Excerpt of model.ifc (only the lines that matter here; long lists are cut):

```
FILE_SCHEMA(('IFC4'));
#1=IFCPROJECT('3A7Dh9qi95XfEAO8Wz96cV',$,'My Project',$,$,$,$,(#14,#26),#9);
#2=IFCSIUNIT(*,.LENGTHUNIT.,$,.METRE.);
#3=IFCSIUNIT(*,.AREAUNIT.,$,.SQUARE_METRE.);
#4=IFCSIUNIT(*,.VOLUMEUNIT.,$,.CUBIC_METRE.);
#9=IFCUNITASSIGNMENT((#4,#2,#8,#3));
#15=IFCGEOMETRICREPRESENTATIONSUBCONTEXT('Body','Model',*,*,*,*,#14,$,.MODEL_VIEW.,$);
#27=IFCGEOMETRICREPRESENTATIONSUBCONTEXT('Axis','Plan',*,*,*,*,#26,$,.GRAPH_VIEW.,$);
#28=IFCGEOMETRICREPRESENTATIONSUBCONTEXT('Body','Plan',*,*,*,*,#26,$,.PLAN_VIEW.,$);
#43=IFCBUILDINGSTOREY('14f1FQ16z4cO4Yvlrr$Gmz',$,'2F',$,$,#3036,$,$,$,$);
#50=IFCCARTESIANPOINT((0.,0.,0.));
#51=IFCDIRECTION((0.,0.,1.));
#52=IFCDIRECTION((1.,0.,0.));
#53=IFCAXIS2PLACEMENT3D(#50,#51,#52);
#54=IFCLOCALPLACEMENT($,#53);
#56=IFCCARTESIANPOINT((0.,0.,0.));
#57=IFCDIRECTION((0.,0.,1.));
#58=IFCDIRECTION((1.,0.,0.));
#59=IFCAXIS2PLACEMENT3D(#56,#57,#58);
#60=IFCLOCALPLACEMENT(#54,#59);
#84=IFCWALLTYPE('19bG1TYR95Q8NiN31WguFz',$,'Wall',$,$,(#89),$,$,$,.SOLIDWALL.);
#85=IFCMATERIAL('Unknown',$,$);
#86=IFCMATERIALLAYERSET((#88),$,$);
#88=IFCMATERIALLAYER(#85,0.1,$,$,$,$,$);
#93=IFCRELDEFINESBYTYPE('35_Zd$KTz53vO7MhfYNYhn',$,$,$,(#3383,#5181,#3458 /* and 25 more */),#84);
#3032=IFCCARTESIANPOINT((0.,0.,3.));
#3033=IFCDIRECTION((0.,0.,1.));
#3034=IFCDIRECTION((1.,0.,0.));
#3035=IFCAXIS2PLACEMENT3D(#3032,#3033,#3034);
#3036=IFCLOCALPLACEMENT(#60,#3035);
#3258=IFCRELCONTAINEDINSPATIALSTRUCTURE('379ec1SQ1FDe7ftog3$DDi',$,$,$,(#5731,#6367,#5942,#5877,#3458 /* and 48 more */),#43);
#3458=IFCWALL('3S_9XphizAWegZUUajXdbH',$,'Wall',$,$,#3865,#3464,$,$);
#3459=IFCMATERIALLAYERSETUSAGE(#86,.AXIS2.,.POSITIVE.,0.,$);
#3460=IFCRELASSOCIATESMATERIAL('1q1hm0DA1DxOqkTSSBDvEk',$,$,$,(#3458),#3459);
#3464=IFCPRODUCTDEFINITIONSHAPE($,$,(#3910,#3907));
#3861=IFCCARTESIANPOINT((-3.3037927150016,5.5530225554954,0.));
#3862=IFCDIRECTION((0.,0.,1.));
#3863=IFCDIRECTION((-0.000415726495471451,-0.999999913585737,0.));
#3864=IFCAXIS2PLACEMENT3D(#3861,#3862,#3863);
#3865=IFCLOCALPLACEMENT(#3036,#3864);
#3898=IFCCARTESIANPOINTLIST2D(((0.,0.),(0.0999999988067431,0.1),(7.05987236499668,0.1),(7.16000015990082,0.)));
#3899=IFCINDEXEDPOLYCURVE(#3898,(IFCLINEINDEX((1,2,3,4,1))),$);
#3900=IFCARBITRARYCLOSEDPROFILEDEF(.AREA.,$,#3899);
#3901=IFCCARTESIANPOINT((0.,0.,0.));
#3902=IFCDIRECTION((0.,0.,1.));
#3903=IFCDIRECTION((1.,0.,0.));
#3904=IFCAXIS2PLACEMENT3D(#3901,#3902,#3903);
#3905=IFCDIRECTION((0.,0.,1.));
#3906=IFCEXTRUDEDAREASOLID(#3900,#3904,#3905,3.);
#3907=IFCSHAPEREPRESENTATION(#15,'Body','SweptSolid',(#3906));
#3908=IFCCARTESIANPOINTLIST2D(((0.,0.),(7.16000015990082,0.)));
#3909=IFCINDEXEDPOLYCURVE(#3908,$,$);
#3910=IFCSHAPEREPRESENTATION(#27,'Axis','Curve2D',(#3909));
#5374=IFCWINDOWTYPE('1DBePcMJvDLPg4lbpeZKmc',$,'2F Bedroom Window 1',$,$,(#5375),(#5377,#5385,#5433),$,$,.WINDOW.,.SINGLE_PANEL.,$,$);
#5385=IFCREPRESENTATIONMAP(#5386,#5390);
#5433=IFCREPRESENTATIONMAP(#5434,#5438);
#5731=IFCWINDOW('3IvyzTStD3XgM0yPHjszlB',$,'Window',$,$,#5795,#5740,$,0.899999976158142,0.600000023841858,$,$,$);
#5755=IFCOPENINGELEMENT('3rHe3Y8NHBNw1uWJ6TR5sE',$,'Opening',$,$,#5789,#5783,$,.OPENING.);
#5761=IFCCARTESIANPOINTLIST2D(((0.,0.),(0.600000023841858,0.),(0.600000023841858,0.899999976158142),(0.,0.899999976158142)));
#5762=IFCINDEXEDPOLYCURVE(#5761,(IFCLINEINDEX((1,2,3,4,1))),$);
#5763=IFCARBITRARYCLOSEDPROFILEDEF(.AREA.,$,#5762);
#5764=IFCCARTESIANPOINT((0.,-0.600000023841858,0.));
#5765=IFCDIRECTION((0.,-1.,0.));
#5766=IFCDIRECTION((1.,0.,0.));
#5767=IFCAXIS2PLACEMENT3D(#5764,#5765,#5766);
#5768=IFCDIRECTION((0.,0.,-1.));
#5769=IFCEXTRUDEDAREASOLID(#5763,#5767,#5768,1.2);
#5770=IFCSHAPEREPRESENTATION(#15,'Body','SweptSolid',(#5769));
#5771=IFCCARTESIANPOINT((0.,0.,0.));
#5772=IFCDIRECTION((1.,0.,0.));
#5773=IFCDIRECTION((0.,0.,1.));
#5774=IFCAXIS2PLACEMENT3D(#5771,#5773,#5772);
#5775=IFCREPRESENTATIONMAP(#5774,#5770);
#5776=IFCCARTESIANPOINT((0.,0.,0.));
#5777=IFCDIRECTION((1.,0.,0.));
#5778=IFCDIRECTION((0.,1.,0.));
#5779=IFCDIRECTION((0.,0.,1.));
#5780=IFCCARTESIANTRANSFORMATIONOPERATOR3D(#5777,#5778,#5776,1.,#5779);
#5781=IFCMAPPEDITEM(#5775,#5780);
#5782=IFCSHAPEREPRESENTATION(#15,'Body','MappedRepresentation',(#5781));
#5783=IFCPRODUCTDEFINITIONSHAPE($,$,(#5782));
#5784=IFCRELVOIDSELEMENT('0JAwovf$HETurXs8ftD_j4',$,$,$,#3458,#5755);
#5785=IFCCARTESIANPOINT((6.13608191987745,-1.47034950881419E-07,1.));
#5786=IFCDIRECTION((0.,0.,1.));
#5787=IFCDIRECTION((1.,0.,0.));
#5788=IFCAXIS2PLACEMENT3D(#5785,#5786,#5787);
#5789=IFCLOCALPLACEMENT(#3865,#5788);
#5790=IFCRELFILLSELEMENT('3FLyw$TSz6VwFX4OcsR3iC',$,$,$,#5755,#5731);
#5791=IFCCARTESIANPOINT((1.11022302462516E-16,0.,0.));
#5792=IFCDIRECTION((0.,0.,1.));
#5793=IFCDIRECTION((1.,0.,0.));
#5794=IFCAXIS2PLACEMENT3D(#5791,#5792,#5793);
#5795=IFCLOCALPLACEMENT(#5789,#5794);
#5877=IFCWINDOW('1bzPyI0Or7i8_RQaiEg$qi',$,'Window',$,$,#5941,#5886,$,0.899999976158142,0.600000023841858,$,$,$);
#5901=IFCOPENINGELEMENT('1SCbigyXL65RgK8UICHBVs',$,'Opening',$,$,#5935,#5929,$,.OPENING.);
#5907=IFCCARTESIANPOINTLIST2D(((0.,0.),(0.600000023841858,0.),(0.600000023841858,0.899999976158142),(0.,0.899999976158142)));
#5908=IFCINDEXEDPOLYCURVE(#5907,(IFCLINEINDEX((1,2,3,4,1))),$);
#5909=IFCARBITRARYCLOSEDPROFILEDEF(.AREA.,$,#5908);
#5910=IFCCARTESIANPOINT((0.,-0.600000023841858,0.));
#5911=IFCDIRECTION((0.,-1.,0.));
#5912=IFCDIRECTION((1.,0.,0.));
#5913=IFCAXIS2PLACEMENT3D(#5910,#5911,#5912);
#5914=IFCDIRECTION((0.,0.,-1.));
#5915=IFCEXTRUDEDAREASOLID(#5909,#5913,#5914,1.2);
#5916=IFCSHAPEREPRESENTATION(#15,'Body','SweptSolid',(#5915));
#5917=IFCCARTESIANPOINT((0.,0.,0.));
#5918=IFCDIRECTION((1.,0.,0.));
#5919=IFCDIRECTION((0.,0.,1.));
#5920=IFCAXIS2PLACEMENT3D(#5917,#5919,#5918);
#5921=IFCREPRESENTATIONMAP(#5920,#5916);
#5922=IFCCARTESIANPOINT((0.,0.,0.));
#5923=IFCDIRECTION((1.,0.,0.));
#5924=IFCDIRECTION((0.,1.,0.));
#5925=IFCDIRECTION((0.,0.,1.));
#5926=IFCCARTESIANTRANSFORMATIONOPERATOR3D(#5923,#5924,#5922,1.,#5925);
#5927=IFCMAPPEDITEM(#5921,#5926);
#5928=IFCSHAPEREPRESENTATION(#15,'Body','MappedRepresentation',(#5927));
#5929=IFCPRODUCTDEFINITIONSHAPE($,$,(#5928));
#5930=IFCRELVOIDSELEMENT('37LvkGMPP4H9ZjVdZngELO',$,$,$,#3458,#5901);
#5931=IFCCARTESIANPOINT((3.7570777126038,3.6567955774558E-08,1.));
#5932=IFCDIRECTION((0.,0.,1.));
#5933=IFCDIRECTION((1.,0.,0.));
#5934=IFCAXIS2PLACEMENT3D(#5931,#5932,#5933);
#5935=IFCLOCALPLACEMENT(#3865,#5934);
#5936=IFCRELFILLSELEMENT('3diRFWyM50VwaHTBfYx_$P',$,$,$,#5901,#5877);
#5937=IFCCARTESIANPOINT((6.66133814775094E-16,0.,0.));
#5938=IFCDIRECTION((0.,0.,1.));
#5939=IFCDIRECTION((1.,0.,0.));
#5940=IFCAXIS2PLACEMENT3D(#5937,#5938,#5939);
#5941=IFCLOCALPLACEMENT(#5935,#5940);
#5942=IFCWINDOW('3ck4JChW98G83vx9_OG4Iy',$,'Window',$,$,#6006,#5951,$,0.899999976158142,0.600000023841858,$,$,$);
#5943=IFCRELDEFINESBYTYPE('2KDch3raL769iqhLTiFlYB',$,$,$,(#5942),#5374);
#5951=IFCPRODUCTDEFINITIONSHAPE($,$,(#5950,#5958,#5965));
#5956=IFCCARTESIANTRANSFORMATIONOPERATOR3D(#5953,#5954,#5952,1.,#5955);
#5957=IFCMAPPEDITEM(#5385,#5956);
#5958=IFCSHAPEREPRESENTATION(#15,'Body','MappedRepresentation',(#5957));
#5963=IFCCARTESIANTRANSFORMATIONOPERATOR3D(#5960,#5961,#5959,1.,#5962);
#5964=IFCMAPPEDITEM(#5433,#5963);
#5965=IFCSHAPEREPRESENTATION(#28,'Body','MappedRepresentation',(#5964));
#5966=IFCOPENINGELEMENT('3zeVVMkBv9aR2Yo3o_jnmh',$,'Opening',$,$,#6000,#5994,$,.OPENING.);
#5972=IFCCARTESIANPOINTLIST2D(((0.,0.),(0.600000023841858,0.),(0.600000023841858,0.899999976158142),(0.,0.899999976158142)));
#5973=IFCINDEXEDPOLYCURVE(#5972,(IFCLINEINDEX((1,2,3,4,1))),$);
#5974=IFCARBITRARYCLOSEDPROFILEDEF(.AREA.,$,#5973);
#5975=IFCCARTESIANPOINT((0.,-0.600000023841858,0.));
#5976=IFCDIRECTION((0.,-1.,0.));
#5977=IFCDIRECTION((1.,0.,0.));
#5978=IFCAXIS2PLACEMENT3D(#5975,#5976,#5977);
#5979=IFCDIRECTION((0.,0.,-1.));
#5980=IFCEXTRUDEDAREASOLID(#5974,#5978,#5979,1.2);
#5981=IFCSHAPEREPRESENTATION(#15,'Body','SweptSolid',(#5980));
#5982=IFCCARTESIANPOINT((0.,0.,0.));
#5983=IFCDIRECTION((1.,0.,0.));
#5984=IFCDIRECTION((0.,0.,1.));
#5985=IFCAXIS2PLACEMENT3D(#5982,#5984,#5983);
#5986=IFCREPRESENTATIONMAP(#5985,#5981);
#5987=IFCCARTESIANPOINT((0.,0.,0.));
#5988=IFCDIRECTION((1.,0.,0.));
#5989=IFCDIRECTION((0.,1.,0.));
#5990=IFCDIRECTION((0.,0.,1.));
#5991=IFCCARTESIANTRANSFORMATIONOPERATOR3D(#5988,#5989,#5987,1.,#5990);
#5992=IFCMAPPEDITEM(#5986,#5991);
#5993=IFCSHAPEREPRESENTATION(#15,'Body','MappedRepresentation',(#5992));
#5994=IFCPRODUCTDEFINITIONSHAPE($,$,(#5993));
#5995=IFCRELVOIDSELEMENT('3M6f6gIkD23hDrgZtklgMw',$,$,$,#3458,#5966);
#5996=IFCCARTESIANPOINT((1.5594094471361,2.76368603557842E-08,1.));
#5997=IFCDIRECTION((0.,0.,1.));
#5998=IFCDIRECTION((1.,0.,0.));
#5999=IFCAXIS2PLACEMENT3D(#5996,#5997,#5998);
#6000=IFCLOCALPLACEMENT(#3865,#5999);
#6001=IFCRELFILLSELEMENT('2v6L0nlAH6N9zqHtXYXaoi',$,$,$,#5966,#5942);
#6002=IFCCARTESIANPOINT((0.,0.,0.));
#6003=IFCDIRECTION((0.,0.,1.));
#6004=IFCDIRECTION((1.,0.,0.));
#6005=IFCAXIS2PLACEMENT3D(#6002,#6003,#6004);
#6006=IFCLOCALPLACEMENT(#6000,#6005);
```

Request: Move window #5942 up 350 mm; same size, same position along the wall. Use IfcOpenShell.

```python
import numpy as np
import ifcopenshell
import ifcopenshell.api.geometry
import ifcopenshell.util.placement
import ifcopenshell.util.unit

model = ifcopenshell.open("model.ifc")
unit_scale = ifcopenshell.util.unit.calculate_unit_scale(model)

window = model.by_id(5942)
opening = window.FillsVoids[0].RelatingOpeningElement
dz = 0.35 / unit_scale

shift = np.array([0.0, 0.0, dz])
# The window is placed relative to its opening, so it follows when the opening moves.
matrix = ifcopenshell.util.placement.get_local_placement(opening.ObjectPlacement)
matrix[:3, 3] += shift
ifcopenshell.api.geometry.edit_object_placement(
    model, product=opening, matrix=matrix, is_si=False, should_transform_children=True
)

print(f"moved by {dz * unit_scale:+.3f} m")

model.write("model_updated.ifc")
```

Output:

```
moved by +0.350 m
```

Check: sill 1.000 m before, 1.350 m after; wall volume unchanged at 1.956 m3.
